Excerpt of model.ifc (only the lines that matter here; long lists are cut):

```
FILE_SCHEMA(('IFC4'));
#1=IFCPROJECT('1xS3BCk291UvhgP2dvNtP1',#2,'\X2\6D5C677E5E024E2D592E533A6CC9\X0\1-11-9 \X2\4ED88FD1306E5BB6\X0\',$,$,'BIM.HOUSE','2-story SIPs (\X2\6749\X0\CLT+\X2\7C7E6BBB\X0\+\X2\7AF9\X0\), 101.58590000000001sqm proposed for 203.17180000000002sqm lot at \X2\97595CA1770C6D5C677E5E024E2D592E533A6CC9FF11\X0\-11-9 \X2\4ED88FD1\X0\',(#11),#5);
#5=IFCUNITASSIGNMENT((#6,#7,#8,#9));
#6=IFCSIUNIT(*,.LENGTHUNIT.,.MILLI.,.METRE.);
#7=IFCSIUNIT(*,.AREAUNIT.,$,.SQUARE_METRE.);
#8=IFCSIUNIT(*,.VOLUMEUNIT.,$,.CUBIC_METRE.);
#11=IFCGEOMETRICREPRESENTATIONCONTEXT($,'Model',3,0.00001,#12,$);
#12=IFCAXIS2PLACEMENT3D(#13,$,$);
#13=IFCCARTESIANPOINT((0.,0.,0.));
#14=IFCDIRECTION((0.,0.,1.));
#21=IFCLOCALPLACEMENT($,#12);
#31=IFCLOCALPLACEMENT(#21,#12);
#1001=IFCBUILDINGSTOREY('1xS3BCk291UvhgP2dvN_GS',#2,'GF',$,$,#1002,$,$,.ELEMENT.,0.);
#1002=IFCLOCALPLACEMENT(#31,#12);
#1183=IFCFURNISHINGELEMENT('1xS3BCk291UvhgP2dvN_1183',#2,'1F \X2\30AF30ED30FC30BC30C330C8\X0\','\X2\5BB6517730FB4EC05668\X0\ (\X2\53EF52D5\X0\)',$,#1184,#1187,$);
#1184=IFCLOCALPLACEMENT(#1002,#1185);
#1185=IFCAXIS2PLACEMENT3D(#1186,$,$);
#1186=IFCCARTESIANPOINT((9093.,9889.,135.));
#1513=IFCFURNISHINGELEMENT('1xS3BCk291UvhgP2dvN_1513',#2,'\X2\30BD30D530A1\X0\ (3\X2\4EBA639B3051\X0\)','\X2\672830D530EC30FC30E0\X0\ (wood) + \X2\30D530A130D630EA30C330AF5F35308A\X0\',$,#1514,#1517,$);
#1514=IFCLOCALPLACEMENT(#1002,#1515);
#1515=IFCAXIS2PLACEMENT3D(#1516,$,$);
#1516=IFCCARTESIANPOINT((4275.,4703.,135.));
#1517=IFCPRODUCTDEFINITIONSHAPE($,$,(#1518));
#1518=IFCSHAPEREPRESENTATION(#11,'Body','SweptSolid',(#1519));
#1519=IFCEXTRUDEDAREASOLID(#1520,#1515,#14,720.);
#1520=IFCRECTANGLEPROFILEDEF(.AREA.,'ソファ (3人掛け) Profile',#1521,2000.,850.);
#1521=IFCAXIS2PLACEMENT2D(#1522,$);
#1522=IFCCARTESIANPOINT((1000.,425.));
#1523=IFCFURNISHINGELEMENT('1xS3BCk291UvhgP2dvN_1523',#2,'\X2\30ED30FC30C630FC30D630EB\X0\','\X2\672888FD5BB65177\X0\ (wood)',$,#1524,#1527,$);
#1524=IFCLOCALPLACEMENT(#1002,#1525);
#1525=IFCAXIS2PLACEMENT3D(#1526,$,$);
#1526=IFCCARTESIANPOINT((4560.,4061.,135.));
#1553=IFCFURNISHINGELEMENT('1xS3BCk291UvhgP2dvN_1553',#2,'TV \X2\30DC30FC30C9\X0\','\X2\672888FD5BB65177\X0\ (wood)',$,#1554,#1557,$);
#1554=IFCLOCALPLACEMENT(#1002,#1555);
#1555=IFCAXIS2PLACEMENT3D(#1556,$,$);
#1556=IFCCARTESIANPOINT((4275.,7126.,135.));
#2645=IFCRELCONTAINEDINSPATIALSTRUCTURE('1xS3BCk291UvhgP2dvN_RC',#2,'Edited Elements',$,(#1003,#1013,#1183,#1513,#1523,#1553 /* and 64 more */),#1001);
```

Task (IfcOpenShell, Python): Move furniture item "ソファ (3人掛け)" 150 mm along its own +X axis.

```python
import ifcopenshell
import ifcopenshell.api.geometry
import ifcopenshell.util.placement
import ifcopenshell.util.unit

model = ifcopenshell.open("model.ifc")
unit_scale = ifcopenshell.util.unit.calculate_unit_scale(model)

item = model.by_guid("1xS3BCk291UvhgP2dvN_1513")
matrix = ifcopenshell.util.placement.get_local_placement(item.ObjectPlacement)
matrix[:3, 3] += matrix[:3, 0] * 0.15 / unit_scale
ifcopenshell.api.geometry.edit_object_placement(model, product=item, matrix=matrix, is_si=False)

print(ifcopenshell.util.placement.get_local_placement(item.ObjectPlacement).round(3) + 0.0)

model.write("model_edited.ifc")
```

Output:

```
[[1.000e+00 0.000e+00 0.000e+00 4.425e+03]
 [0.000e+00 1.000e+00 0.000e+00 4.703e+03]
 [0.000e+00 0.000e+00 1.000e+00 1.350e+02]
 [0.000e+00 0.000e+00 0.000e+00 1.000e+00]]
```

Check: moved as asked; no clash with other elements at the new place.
